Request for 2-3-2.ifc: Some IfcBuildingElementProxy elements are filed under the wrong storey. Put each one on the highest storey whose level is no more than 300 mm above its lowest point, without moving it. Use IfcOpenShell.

First a look at what the model holds.

```python
import ifcopenshell
import ifcopenshell.util.element
import ifcopenshell.util.placement

model = ifcopenshell.open("2-3-2.ifc")
print(model.schema)
for storey in model.by_type("IfcBuildingStorey"):
    level = ifcopenshell.util.placement.get_storey_elevation(storey)
    count = sum(e.is_a("IfcBuildingElementProxy") for e in ifcopenshell.util.element.get_contained(storey))
    print(storey.id(), storey.Name, round(level, 3), count, sep=" | ")
```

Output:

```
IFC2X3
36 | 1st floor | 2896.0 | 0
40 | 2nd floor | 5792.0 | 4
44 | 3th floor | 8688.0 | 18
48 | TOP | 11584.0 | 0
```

```python
import ifcopenshell
import ifcopenshell.api.spatial
import ifcopenshell.geom
import ifcopenshell.util.element
import ifcopenshell.util.placement
import ifcopenshell.util.shape
import ifcopenshell.util.unit

model = ifcopenshell.open("2-3-2.ifc")
unit_scale = ifcopenshell.util.unit.calculate_unit_scale(model)
settings = ifcopenshell.geom.settings()

levels = sorted(
    ((ifcopenshell.util.placement.get_storey_elevation(s) * unit_scale, s) for s in model.by_type("IfcBuildingStorey")),
    key=lambda pair: pair[0],
)

for e in model.by_type("IfcBuildingElementProxy"):
    current = e.ContainedInStructure[0].RelatingStructure if e.ContainedInStructure else None
    if current is None or not current.is_a("IfcBuildingStorey"):
        continue
    shape = ifcopenshell.geom.create_shape(settings, e)
    bottom = ifcopenshell.util.shape.get_shape_bottom_elevation(shape, shape.geometry)
    below = [s for level, s in levels if level <= bottom + 0.3]
    storey = below[-1] if below else levels[0][1]
    if storey != current:
        # assign_container keeps the world position.
        ifcopenshell.api.spatial.assign_container(model, products=[e], relating_structure=storey)
        print(e.id(), current.Name, "->", storey.Name)

model.write("2-3-2_updated.ifc")
```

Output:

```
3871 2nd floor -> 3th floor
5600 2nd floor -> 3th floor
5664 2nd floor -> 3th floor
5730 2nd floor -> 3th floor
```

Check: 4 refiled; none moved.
